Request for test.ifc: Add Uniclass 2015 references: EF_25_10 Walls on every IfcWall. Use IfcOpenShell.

First a look at what the model holds.

```python
import ifcopenshell

model = ifcopenshell.open("test.ifc")
print(model.schema)
print("classifications:", [c.Name for c in model.by_type("IfcClassification")])
for ifc_class in ("IfcDoor", "IfcRoof", "IfcStair", "IfcWall", "IfcWindow"):
    print(ifc_class, len(model.by_type(ifc_class)))
```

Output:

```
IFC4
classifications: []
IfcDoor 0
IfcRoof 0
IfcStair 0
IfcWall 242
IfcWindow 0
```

```python
import ifcopenshell
import ifcopenshell.api.classification

model = ifcopenshell.open("test.ifc")

system = ifcopenshell.api.classification.add_classification(model, classification="Uniclass 2015")

codes = {
    "IfcWall": ("EF_25_10", "Walls"),
}
for ifc_class, (code, name) in codes.items():
    products = model.by_type(ifc_class)
    ifcopenshell.api.classification.add_reference(
        model, products=products, classification=system, identification=code, name=name
    )
    print(code, len(products))

model.write("test-out.ifc")
```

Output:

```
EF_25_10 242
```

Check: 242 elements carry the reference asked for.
